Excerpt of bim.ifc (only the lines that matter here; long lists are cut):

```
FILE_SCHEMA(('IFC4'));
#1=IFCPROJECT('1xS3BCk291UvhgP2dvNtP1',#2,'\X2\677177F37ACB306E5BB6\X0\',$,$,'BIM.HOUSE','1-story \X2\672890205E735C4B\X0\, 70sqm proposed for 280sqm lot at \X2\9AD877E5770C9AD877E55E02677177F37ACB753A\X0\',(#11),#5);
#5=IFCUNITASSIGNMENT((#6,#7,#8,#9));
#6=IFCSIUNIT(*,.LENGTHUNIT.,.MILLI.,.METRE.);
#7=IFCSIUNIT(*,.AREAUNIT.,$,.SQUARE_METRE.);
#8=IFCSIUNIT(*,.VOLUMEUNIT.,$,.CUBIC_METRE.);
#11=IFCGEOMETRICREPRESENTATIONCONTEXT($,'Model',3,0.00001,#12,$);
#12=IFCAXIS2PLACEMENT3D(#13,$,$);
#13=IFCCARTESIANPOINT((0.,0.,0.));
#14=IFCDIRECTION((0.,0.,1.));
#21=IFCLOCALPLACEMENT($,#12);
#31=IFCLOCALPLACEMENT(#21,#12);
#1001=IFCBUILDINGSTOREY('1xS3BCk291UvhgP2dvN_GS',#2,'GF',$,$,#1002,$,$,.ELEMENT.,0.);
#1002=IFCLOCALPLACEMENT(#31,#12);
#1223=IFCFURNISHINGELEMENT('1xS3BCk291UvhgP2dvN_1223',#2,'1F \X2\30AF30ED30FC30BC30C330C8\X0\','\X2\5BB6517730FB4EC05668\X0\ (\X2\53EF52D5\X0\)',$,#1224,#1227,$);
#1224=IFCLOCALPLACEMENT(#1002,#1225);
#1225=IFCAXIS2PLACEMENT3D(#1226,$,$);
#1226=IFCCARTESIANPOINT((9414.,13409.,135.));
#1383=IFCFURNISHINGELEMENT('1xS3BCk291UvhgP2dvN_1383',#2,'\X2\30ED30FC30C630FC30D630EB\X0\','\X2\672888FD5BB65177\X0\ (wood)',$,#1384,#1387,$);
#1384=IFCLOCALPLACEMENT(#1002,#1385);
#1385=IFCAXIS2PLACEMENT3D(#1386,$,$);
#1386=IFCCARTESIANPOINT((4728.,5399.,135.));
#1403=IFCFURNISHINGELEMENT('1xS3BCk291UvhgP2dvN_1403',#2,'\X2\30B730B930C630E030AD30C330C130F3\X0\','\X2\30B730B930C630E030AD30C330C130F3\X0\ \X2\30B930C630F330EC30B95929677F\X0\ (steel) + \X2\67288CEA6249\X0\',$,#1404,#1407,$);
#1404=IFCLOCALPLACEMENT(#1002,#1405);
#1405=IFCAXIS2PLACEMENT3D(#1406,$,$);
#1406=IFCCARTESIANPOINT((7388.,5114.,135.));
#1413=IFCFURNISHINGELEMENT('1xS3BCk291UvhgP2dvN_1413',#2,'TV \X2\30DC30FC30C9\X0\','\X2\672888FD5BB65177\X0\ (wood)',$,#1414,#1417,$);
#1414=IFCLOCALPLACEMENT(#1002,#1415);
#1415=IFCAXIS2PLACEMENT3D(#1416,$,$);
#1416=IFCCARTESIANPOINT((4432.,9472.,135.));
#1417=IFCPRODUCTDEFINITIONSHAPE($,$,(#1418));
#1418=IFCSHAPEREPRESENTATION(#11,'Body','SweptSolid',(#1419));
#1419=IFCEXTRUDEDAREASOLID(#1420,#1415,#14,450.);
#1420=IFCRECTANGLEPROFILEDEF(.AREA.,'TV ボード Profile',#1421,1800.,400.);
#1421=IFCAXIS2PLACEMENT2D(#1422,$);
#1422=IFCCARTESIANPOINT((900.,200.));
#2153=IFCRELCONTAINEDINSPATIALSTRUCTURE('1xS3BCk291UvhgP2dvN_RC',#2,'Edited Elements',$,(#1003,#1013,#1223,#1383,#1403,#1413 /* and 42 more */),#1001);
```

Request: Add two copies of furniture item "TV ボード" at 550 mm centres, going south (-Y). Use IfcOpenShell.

```python
import numpy as np
import ifcopenshell
import ifcopenshell.api.geometry
import ifcopenshell.api.root
import ifcopenshell.util.element
import ifcopenshell.util.placement
import ifcopenshell.util.unit

model = ifcopenshell.open("bim.ifc")
unit_scale = ifcopenshell.util.unit.calculate_unit_scale(model)


def reuse_history(source, copy):
    """copy_class also copies each property set's owner history, people and application; keep the originals."""
    for rel in copy.IsDefinedBy:
        if rel.is_a("IfcRelDefinesByProperties") and (history := rel.RelatingPropertyDefinition.OwnerHistory):
            rel.RelatingPropertyDefinition.OwnerHistory = source.OwnerHistory
            ifcopenshell.util.element.remove_deep2(model, history)


source = model.by_guid("1xS3BCk291UvhgP2dvN_1413")
base = ifcopenshell.util.placement.get_local_placement(source.ObjectPlacement)
step = np.array([0.0, -1.0, 0.0]) * 0.55 / unit_scale

for i in range(1, 3):
    copy = ifcopenshell.api.root.copy_class(model, product=source)
    copy.Representation = ifcopenshell.util.element.copy_deep(
        model, source.Representation, exclude=["IfcGeometricRepresentationContext", "IfcRepresentationMap"]
    )
    reuse_history(source, copy)
    matrix = base.copy()
    matrix[:3, 3] += i * step
    print("added at", matrix[:3, 3].round(3) + 0.0)
    ifcopenshell.api.geometry.edit_object_placement(model, product=copy, matrix=matrix, is_si=False)

model.write("bim_edited.ifc")
```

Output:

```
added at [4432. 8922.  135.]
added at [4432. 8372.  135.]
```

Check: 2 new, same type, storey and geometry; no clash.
